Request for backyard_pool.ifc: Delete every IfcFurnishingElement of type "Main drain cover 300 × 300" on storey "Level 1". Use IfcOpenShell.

First a look at what the model holds.

```python
import ifcopenshell
import ifcopenshell.util.element

model = ifcopenshell.open("backyard_pool.ifc")
print(model.schema)
storey = next(s for s in model.by_type("IfcBuildingStorey") if s.Name == "Level 1")
furniture = [e for e in ifcopenshell.util.element.get_decomposition(storey) if e.is_a("IfcFurnishingElement")]
seen = {}
for e in furniture:
    element_type = ifcopenshell.util.element.get_type(e)
    name = element_type.Name if element_type not in (None, e) else None
    seen[name] = seen.get(name, 0) + 1
for name, count in sorted(seen.items(), key=str):
    print(count, "x", name)
```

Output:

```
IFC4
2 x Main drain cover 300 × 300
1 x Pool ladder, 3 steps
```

```python
import ifcopenshell
import ifcopenshell.api.root
import ifcopenshell.util.element

model = ifcopenshell.open("backyard_pool.ifc")

storey = next(s for s in model.by_type("IfcBuildingStorey") if s.Name == "Level 1")
furniture = [e for e in ifcopenshell.util.element.get_decomposition(storey) if e.is_a("IfcFurnishingElement")]
targets = [e for e in furniture if (t := ifcopenshell.util.element.get_type(e)) not in (None, e) and t.Name == "Main drain cover 300 × 300"]

for e in targets:
    ifcopenshell.api.root.remove_product(model, product=e)
print(len(targets), "removed")

model.write("backyard_pool-out.ifc")
```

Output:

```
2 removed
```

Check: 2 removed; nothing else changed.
